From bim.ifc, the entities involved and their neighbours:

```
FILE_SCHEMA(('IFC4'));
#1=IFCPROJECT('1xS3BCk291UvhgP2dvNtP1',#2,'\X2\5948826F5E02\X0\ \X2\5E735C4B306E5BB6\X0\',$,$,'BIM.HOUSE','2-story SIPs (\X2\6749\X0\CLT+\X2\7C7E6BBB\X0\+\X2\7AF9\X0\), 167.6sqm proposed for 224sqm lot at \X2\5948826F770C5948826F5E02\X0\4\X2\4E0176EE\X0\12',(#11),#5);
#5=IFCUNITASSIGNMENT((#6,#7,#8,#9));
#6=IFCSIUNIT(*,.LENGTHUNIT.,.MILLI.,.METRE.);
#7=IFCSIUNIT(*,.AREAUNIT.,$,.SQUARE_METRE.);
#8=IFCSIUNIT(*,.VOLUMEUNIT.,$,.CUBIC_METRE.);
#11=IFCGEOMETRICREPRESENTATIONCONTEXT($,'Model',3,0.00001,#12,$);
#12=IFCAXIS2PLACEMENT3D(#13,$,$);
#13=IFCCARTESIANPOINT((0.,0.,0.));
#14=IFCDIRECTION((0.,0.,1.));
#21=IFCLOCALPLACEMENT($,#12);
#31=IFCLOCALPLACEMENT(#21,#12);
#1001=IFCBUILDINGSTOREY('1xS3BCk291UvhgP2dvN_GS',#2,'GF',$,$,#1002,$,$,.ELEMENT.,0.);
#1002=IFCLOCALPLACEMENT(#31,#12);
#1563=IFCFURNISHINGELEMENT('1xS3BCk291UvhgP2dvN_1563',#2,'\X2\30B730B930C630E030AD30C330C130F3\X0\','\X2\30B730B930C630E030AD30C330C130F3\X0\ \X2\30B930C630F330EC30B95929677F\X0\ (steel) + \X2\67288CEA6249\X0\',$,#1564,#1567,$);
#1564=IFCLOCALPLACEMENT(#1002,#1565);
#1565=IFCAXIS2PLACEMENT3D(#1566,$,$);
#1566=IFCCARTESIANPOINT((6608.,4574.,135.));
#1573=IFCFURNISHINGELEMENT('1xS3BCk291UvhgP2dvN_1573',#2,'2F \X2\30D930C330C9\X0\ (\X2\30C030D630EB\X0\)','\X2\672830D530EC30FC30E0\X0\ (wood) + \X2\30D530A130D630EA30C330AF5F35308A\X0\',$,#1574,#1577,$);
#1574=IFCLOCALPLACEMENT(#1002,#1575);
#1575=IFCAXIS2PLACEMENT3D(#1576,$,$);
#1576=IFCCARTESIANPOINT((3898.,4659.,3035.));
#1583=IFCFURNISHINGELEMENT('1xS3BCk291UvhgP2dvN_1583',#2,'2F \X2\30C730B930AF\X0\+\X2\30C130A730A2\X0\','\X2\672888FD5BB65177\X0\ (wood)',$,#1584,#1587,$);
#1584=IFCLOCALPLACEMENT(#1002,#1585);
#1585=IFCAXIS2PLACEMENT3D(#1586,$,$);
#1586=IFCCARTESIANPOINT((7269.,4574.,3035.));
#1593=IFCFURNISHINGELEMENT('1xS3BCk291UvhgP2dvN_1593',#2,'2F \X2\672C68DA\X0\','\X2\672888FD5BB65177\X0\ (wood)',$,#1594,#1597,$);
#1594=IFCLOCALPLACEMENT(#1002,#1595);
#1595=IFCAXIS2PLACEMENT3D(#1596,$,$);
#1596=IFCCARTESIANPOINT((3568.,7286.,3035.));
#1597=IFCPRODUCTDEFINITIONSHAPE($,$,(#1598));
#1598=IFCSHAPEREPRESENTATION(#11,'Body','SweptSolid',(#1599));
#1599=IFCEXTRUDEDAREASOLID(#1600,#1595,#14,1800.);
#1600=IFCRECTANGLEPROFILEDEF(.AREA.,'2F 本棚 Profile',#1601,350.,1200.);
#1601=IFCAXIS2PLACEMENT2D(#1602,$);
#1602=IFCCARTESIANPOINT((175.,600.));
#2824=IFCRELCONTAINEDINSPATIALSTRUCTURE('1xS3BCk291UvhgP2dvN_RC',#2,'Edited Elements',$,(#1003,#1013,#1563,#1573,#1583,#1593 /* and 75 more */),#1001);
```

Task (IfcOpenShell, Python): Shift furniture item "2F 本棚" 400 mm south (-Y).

```python
import ifcopenshell
import ifcopenshell.api.geometry
import ifcopenshell.util.placement
import ifcopenshell.util.unit

model = ifcopenshell.open("bim.ifc")
unit_scale = ifcopenshell.util.unit.calculate_unit_scale(model)

item = model.by_guid("1xS3BCk291UvhgP2dvN_1593")
matrix = ifcopenshell.util.placement.get_local_placement(item.ObjectPlacement)
matrix[1, 3] -= 0.4 / unit_scale
ifcopenshell.api.geometry.edit_object_placement(model, product=item, matrix=matrix, is_si=False)

print(ifcopenshell.util.placement.get_local_placement(item.ObjectPlacement).round(3) + 0.0)

model.write("bim_updated.ifc")
```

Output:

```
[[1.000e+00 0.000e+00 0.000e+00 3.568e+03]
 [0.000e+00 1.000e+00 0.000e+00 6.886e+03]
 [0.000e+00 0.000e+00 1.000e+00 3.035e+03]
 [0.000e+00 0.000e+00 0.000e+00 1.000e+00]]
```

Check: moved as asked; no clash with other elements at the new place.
